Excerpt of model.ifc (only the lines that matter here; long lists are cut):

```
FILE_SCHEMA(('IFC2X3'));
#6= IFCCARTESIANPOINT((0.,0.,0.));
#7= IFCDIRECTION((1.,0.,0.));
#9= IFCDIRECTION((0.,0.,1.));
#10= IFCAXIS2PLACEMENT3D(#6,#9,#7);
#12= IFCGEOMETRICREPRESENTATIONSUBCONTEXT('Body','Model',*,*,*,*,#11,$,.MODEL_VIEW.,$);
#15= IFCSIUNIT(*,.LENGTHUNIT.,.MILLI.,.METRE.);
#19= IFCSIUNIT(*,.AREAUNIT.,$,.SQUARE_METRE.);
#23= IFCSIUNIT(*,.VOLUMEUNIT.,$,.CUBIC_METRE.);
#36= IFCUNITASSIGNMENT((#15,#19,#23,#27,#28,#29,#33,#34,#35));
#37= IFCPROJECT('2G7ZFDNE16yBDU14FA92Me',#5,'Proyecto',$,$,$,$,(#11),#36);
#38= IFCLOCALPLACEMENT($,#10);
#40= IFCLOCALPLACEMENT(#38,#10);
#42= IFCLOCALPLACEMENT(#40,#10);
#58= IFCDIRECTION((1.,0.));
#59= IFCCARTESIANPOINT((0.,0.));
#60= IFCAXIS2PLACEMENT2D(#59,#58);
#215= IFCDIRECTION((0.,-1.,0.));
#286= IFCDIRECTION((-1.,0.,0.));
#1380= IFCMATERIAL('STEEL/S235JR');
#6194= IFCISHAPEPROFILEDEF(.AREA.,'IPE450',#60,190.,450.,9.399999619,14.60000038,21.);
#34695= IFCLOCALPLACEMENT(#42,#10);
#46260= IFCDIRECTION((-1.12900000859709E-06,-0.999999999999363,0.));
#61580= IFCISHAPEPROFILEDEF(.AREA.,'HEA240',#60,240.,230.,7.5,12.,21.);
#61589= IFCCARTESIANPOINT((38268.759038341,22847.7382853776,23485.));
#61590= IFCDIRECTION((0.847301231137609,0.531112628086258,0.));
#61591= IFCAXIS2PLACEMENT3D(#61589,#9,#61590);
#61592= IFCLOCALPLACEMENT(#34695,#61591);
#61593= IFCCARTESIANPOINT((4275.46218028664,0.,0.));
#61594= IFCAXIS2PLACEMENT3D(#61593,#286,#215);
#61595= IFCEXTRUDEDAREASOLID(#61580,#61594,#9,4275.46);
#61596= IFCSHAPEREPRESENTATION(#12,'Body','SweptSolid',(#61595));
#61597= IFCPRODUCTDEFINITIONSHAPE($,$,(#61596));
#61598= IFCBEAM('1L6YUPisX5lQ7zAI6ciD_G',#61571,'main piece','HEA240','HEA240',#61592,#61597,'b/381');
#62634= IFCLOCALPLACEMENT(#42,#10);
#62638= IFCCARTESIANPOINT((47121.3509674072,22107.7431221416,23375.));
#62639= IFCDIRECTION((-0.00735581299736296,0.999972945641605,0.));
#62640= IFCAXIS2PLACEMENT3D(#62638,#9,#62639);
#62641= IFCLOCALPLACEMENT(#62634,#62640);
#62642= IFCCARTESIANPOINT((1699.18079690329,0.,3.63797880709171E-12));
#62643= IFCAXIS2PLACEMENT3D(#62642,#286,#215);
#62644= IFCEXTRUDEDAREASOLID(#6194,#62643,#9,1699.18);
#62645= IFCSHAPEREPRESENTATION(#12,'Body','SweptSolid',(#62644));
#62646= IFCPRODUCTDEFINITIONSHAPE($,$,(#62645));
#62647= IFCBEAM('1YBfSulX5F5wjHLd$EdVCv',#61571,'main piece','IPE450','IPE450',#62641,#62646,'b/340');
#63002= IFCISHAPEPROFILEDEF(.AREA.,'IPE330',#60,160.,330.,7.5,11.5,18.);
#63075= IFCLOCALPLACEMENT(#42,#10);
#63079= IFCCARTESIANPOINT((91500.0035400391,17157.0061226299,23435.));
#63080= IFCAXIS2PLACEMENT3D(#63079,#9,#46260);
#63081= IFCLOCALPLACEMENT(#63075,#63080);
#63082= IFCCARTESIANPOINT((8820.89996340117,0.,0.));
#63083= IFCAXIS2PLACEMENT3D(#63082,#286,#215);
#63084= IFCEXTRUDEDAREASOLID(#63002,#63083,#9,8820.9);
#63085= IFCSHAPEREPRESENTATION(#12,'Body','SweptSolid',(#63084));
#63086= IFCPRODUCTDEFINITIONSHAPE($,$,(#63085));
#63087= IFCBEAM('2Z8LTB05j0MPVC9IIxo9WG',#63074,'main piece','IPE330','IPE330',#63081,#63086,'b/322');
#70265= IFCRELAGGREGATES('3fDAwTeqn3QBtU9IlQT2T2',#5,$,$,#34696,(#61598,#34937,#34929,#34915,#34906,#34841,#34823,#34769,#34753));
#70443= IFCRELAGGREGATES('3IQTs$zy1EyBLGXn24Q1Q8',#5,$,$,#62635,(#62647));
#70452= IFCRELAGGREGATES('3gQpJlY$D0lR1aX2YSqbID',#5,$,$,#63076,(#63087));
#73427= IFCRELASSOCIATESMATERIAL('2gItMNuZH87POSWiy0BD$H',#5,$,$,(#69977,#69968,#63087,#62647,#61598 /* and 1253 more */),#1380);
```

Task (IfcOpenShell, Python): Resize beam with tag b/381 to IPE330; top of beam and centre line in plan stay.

```python
import ifcopenshell
import ifcopenshell.util.element
import ifcopenshell.util.representation

model = ifcopenshell.open("model.ifc")

member = model.by_guid("1L6YUPisX5lQ7zAI6ciD_G")
source = next(p for p in model.by_type("IfcIShapeProfileDef") if p.ProfileName == "IPE330")

body = ifcopenshell.util.representation.get_representation(member, "Model", "Body")
solid = body.Items[0]
old_profile = solid.SweptArea

# Copy the section's sizes but keep this member's own profile position.
profile = ifcopenshell.util.element.copy(model, source)
# Profiles are centred, so shift by half the change in depth to hold the top.
shift = (old_profile.OverallDepth - profile.OverallDepth) / 2
x, y = old_profile.Position.Location.Coordinates
up = (0.0, 1.0)  # upwards, in the solid's own plane
location = model.createIfcCartesianPoint((x + up[0] * shift, y + up[1] * shift))
profile.Position = model.createIfcAxis2Placement2D(location, old_profile.Position.RefDirection)
solid.SweptArea = profile
if not model.get_total_inverses(old_profile):
    ifcopenshell.util.element.remove_deep2(model, old_profile)
member.Description = member.Description.replace("HEA240", "IPE330")
member.ObjectType = member.ObjectType.replace("HEA240", "IPE330")

print(solid.SweptArea)

model.write("model_v2.ifc")
```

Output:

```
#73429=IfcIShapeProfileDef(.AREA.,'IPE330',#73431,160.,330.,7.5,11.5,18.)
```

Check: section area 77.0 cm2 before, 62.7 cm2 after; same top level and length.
